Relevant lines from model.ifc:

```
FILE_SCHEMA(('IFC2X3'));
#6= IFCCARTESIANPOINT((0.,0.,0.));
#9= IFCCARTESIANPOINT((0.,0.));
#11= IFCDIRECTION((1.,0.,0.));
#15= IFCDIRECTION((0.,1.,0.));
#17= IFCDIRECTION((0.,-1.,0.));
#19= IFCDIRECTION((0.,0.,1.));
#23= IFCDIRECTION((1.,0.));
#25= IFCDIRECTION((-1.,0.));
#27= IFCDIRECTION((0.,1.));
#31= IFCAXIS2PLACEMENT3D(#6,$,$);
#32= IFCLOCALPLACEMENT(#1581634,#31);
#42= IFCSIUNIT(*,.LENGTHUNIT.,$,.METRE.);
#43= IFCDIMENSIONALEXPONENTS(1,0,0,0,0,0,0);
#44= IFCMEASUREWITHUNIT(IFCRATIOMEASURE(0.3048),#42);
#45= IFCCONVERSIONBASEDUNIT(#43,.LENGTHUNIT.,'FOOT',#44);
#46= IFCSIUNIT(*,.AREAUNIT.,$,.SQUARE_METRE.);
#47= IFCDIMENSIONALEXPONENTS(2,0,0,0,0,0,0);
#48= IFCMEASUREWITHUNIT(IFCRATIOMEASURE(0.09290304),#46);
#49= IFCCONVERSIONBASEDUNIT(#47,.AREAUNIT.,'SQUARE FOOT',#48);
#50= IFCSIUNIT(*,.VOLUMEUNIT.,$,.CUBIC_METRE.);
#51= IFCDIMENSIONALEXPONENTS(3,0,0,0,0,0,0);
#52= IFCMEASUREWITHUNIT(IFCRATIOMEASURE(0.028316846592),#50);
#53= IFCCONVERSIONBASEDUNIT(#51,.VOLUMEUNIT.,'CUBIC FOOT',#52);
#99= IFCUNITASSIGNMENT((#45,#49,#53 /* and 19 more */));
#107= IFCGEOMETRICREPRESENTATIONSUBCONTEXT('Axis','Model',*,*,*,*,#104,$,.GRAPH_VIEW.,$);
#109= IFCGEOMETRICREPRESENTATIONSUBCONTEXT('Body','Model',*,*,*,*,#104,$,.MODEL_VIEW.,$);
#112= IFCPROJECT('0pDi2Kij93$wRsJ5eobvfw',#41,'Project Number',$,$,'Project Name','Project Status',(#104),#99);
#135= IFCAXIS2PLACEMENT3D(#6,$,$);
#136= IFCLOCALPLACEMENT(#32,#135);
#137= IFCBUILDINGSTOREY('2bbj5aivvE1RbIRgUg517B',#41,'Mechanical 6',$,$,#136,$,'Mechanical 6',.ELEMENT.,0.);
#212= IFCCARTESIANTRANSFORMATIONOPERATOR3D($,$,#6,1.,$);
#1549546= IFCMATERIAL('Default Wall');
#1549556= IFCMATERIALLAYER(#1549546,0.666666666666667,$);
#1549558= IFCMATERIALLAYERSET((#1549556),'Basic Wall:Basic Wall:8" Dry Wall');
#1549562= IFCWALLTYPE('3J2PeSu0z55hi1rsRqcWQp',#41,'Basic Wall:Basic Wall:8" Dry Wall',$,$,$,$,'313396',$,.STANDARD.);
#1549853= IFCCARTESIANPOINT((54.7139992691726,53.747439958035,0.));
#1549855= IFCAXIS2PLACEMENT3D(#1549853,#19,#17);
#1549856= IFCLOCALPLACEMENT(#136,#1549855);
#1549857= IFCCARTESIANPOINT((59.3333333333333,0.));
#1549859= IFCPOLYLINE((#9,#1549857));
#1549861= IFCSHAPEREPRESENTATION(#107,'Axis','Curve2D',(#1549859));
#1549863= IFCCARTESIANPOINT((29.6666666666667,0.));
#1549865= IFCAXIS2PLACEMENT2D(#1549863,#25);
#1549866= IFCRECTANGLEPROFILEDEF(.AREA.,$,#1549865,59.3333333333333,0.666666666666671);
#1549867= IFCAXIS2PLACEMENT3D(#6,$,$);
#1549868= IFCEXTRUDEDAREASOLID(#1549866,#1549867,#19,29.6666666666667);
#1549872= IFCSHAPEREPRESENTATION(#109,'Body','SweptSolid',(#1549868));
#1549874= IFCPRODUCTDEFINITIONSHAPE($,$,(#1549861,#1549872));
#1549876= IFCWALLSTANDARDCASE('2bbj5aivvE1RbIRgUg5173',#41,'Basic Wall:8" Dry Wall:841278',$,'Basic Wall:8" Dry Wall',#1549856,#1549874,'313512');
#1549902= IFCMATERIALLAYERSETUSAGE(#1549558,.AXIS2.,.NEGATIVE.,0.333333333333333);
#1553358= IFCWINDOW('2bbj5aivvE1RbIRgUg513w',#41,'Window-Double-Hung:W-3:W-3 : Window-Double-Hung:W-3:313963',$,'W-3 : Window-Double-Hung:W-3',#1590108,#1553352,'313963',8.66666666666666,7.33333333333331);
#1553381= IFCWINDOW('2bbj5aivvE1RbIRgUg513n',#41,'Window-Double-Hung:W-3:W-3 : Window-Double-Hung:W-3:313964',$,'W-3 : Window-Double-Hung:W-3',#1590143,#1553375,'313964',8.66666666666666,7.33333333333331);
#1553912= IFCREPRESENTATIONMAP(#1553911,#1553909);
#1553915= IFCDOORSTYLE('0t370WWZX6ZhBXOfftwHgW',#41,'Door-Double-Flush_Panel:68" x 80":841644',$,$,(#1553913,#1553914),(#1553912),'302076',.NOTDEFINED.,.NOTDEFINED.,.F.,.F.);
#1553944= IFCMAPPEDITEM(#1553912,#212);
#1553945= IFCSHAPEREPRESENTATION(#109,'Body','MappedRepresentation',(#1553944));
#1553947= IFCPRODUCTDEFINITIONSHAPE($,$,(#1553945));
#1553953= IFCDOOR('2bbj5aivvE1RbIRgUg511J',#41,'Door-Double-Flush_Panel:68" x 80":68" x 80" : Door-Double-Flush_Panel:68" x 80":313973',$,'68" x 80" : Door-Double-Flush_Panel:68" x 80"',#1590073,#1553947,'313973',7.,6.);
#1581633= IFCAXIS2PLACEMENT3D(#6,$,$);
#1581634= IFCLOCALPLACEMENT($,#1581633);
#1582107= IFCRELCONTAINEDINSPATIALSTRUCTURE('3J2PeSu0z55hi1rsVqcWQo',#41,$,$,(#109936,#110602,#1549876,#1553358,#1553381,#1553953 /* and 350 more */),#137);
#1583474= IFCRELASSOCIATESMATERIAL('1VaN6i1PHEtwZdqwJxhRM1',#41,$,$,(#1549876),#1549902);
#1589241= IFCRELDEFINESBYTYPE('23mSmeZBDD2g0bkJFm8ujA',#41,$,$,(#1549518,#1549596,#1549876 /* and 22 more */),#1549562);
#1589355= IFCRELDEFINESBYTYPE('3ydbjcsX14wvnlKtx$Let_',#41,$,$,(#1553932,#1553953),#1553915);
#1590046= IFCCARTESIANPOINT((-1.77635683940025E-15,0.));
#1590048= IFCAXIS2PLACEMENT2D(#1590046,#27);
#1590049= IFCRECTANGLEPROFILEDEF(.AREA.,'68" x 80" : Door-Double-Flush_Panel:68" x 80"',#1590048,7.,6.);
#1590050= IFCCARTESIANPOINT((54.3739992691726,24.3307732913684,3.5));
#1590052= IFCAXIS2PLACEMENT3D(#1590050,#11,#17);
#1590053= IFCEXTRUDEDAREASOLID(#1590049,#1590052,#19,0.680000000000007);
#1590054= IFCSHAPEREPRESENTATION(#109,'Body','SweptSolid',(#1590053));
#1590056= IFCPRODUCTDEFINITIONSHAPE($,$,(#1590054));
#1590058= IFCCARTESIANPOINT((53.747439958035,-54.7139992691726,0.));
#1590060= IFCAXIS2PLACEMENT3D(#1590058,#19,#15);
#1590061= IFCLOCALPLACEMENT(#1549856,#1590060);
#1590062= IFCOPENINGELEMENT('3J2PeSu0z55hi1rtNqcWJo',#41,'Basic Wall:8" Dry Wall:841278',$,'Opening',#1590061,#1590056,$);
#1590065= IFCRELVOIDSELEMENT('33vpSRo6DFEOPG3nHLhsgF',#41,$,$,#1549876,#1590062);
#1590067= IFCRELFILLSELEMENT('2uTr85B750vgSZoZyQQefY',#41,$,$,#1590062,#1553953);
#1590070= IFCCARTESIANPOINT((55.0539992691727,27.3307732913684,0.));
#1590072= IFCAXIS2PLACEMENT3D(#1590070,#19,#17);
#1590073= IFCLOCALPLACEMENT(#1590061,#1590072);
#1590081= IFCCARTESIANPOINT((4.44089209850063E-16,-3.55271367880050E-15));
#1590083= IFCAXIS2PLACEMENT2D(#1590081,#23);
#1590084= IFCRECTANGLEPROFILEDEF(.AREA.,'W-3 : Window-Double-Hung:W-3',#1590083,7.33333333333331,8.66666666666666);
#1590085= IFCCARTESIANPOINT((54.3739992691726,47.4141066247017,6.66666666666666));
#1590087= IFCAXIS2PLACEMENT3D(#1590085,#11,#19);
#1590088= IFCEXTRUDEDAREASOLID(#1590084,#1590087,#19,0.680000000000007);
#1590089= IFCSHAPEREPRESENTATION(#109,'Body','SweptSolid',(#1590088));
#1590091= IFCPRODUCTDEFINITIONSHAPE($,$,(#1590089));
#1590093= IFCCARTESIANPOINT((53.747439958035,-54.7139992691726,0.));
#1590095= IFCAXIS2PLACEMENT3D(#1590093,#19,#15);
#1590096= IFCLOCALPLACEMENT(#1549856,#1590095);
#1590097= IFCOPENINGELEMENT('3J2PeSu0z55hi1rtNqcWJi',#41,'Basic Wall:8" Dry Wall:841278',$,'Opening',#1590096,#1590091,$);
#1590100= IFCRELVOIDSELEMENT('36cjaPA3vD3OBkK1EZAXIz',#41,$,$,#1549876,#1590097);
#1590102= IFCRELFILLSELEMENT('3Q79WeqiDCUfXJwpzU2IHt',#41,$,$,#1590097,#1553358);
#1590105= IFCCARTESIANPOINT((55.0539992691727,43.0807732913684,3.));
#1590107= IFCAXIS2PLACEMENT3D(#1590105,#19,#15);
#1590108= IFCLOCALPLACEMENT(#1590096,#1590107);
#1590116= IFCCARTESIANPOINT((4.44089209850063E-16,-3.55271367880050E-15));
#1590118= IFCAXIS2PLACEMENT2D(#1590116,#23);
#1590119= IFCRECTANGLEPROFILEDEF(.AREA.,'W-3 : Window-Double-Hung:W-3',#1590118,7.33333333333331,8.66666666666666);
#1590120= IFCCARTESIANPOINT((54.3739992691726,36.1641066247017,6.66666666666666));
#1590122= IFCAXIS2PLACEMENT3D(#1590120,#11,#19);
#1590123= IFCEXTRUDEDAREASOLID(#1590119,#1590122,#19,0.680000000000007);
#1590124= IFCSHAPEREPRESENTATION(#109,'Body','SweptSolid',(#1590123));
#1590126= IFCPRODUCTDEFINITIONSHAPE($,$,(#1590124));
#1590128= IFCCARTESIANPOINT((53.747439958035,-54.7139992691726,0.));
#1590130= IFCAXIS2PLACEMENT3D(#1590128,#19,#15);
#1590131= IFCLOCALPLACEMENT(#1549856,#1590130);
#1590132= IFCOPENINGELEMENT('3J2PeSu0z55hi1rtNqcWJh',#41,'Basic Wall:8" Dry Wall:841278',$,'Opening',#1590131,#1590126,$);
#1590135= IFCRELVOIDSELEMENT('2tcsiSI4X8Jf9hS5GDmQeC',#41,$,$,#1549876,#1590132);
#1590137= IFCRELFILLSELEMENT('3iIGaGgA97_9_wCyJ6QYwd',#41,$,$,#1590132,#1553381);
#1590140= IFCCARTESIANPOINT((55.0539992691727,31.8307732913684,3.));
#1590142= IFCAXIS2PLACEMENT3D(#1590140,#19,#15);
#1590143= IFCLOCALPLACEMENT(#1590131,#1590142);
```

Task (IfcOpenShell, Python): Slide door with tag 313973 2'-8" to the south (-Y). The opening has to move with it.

```python
import ifcopenshell
import ifcopenshell.api.geometry
import ifcopenshell.util.placement
import ifcopenshell.util.unit

model = ifcopenshell.open("model.ifc")
unit_scale = ifcopenshell.util.unit.calculate_unit_scale(model)

door = model.by_guid("2bbj5aivvE1RbIRgUg511J")
opening = door.FillsVoids[0].RelatingOpeningElement
wall = opening.VoidsElements[0].RelatingBuildingElement

wall_matrix = ifcopenshell.util.placement.get_local_placement(wall.ObjectPlacement)
shift = wall_matrix[:3, 0] * 32 * 0.0254 / unit_scale
before = ifcopenshell.util.placement.get_local_placement(door.ObjectPlacement)[:3, 3].copy()

# The door is placed relative to its opening, so it follows when the opening moves.
matrix = ifcopenshell.util.placement.get_local_placement(opening.ObjectPlacement)
matrix[:3, 3] += shift
ifcopenshell.api.geometry.edit_object_placement(
    model, product=opening, matrix=matrix, is_si=False, should_transform_children=True
)

after = ifcopenshell.util.placement.get_local_placement(door.ObjectPlacement)[:3, 3]
print("door moved by", (after - before).round(3) + 0.0)

model.write("model_rev.ifc")
```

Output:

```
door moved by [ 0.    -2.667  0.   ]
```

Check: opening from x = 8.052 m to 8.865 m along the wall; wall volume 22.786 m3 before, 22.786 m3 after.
